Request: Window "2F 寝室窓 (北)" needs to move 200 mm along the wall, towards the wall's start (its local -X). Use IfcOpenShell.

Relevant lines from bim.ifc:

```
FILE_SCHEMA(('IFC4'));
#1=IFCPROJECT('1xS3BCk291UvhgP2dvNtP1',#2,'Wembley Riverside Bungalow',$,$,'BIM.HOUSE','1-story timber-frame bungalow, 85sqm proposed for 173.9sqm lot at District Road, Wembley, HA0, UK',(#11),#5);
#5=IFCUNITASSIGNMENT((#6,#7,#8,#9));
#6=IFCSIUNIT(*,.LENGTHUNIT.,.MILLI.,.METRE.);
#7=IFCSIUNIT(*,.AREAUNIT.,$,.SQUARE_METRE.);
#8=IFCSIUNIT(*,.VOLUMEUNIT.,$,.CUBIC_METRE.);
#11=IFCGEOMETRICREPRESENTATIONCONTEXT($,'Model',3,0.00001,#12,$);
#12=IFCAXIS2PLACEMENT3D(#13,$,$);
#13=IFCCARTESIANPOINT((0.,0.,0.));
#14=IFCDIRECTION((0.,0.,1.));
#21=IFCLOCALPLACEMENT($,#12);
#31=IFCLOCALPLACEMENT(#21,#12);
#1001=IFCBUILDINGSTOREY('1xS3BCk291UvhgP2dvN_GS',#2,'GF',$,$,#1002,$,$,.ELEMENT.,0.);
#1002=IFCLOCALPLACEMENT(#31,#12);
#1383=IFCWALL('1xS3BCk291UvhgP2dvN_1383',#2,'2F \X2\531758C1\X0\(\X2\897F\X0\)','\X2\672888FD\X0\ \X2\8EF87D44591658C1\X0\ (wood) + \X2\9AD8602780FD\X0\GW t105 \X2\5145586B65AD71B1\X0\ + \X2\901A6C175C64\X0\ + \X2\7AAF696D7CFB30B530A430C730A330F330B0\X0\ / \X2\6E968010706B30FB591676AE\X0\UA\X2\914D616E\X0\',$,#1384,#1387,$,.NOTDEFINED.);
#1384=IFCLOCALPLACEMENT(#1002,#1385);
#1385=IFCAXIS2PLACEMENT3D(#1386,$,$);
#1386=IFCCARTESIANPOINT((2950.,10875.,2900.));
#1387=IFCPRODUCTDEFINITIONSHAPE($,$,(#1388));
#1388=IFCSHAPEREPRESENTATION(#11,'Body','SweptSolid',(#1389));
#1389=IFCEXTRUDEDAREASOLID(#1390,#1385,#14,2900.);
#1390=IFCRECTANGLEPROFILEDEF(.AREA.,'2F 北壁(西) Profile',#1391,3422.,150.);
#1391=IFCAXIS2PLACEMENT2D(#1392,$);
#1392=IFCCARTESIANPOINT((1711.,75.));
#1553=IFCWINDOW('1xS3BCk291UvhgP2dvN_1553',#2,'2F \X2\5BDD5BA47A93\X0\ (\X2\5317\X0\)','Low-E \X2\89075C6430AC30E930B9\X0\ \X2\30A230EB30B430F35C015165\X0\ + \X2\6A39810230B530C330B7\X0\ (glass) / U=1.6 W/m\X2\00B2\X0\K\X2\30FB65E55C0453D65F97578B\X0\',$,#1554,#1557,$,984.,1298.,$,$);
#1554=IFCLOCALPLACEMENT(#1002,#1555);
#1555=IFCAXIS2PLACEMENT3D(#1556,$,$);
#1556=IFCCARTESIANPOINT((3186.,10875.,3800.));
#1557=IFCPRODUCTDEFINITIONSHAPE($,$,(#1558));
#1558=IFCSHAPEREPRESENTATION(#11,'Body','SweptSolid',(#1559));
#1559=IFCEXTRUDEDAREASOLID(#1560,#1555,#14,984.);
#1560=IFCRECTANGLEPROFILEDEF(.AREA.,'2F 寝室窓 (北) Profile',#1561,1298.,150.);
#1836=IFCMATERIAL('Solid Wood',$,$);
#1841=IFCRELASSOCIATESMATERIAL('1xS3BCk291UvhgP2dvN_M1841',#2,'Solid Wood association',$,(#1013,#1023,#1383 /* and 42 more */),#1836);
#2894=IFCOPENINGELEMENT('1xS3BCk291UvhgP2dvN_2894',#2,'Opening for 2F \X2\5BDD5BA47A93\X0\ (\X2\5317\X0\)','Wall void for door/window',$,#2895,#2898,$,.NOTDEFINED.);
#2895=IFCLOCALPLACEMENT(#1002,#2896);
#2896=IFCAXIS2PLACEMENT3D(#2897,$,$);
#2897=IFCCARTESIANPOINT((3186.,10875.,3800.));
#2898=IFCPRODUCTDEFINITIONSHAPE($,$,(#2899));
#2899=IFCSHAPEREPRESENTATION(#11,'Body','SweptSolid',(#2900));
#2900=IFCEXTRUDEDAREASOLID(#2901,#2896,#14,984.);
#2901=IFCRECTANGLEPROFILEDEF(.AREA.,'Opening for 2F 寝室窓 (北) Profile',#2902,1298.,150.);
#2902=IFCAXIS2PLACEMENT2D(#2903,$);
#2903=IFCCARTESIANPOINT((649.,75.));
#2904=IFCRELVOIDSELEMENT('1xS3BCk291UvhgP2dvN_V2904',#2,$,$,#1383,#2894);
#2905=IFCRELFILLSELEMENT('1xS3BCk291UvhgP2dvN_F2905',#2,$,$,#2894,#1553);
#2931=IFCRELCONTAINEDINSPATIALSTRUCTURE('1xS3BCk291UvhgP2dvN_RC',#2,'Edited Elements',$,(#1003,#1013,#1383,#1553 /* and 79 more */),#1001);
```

```python
import ifcopenshell
import ifcopenshell.api.geometry
import ifcopenshell.util.placement
import ifcopenshell.util.unit

model = ifcopenshell.open("bim.ifc")
unit_scale = ifcopenshell.util.unit.calculate_unit_scale(model)

window = model.by_guid("1xS3BCk291UvhgP2dvN_1553")
opening = window.FillsVoids[0].RelatingOpeningElement
wall = opening.VoidsElements[0].RelatingBuildingElement

wall_matrix = ifcopenshell.util.placement.get_local_placement(wall.ObjectPlacement)
shift = wall_matrix[:3, 0] * -0.2 / unit_scale
before = ifcopenshell.util.placement.get_local_placement(window.ObjectPlacement)[:3, 3].copy()

# The window is not placed relative to its opening, so move both.
for product in (opening, window):
    matrix = ifcopenshell.util.placement.get_local_placement(product.ObjectPlacement)
    matrix[:3, 3] += shift
    ifcopenshell.api.geometry.edit_object_placement(model, product=product, matrix=matrix, is_si=False)

after = ifcopenshell.util.placement.get_local_placement(window.ObjectPlacement)[:3, 3]
print("window moved by", (after - before).round(3) + 0.0)

model.write("bim_edited.ifc")
```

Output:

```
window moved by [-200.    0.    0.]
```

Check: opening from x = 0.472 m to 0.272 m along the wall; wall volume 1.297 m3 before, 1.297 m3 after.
